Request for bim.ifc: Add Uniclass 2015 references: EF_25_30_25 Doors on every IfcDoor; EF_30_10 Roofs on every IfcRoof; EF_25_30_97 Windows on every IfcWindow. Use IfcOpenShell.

First a look at what the model holds.

```python
import ifcopenshell

model = ifcopenshell.open("bim.ifc")
print(model.schema)
print("classifications:", [c.Name for c in model.by_type("IfcClassification")])
for ifc_class in ("IfcDoor", "IfcRoof", "IfcStair", "IfcWall", "IfcWindow"):
    print(ifc_class, len(model.by_type(ifc_class)))
```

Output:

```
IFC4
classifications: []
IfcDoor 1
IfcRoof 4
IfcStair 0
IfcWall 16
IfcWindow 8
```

```python
import ifcopenshell
import ifcopenshell.api.classification

model = ifcopenshell.open("bim.ifc")

system = ifcopenshell.api.classification.add_classification(model, classification="Uniclass 2015")

codes = {
    "IfcDoor": ("EF_25_30_25", "Doors"),
    "IfcRoof": ("EF_30_10", "Roofs"),
    "IfcWindow": ("EF_25_30_97", "Windows"),
}
for ifc_class, (code, name) in codes.items():
    products = model.by_type(ifc_class)
    ifcopenshell.api.classification.add_reference(
        model, products=products, classification=system, identification=code, name=name
    )
    print(code, len(products))

model.write("bim_updated.ifc")
```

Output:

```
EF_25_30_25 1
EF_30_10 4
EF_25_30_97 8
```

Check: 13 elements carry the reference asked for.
